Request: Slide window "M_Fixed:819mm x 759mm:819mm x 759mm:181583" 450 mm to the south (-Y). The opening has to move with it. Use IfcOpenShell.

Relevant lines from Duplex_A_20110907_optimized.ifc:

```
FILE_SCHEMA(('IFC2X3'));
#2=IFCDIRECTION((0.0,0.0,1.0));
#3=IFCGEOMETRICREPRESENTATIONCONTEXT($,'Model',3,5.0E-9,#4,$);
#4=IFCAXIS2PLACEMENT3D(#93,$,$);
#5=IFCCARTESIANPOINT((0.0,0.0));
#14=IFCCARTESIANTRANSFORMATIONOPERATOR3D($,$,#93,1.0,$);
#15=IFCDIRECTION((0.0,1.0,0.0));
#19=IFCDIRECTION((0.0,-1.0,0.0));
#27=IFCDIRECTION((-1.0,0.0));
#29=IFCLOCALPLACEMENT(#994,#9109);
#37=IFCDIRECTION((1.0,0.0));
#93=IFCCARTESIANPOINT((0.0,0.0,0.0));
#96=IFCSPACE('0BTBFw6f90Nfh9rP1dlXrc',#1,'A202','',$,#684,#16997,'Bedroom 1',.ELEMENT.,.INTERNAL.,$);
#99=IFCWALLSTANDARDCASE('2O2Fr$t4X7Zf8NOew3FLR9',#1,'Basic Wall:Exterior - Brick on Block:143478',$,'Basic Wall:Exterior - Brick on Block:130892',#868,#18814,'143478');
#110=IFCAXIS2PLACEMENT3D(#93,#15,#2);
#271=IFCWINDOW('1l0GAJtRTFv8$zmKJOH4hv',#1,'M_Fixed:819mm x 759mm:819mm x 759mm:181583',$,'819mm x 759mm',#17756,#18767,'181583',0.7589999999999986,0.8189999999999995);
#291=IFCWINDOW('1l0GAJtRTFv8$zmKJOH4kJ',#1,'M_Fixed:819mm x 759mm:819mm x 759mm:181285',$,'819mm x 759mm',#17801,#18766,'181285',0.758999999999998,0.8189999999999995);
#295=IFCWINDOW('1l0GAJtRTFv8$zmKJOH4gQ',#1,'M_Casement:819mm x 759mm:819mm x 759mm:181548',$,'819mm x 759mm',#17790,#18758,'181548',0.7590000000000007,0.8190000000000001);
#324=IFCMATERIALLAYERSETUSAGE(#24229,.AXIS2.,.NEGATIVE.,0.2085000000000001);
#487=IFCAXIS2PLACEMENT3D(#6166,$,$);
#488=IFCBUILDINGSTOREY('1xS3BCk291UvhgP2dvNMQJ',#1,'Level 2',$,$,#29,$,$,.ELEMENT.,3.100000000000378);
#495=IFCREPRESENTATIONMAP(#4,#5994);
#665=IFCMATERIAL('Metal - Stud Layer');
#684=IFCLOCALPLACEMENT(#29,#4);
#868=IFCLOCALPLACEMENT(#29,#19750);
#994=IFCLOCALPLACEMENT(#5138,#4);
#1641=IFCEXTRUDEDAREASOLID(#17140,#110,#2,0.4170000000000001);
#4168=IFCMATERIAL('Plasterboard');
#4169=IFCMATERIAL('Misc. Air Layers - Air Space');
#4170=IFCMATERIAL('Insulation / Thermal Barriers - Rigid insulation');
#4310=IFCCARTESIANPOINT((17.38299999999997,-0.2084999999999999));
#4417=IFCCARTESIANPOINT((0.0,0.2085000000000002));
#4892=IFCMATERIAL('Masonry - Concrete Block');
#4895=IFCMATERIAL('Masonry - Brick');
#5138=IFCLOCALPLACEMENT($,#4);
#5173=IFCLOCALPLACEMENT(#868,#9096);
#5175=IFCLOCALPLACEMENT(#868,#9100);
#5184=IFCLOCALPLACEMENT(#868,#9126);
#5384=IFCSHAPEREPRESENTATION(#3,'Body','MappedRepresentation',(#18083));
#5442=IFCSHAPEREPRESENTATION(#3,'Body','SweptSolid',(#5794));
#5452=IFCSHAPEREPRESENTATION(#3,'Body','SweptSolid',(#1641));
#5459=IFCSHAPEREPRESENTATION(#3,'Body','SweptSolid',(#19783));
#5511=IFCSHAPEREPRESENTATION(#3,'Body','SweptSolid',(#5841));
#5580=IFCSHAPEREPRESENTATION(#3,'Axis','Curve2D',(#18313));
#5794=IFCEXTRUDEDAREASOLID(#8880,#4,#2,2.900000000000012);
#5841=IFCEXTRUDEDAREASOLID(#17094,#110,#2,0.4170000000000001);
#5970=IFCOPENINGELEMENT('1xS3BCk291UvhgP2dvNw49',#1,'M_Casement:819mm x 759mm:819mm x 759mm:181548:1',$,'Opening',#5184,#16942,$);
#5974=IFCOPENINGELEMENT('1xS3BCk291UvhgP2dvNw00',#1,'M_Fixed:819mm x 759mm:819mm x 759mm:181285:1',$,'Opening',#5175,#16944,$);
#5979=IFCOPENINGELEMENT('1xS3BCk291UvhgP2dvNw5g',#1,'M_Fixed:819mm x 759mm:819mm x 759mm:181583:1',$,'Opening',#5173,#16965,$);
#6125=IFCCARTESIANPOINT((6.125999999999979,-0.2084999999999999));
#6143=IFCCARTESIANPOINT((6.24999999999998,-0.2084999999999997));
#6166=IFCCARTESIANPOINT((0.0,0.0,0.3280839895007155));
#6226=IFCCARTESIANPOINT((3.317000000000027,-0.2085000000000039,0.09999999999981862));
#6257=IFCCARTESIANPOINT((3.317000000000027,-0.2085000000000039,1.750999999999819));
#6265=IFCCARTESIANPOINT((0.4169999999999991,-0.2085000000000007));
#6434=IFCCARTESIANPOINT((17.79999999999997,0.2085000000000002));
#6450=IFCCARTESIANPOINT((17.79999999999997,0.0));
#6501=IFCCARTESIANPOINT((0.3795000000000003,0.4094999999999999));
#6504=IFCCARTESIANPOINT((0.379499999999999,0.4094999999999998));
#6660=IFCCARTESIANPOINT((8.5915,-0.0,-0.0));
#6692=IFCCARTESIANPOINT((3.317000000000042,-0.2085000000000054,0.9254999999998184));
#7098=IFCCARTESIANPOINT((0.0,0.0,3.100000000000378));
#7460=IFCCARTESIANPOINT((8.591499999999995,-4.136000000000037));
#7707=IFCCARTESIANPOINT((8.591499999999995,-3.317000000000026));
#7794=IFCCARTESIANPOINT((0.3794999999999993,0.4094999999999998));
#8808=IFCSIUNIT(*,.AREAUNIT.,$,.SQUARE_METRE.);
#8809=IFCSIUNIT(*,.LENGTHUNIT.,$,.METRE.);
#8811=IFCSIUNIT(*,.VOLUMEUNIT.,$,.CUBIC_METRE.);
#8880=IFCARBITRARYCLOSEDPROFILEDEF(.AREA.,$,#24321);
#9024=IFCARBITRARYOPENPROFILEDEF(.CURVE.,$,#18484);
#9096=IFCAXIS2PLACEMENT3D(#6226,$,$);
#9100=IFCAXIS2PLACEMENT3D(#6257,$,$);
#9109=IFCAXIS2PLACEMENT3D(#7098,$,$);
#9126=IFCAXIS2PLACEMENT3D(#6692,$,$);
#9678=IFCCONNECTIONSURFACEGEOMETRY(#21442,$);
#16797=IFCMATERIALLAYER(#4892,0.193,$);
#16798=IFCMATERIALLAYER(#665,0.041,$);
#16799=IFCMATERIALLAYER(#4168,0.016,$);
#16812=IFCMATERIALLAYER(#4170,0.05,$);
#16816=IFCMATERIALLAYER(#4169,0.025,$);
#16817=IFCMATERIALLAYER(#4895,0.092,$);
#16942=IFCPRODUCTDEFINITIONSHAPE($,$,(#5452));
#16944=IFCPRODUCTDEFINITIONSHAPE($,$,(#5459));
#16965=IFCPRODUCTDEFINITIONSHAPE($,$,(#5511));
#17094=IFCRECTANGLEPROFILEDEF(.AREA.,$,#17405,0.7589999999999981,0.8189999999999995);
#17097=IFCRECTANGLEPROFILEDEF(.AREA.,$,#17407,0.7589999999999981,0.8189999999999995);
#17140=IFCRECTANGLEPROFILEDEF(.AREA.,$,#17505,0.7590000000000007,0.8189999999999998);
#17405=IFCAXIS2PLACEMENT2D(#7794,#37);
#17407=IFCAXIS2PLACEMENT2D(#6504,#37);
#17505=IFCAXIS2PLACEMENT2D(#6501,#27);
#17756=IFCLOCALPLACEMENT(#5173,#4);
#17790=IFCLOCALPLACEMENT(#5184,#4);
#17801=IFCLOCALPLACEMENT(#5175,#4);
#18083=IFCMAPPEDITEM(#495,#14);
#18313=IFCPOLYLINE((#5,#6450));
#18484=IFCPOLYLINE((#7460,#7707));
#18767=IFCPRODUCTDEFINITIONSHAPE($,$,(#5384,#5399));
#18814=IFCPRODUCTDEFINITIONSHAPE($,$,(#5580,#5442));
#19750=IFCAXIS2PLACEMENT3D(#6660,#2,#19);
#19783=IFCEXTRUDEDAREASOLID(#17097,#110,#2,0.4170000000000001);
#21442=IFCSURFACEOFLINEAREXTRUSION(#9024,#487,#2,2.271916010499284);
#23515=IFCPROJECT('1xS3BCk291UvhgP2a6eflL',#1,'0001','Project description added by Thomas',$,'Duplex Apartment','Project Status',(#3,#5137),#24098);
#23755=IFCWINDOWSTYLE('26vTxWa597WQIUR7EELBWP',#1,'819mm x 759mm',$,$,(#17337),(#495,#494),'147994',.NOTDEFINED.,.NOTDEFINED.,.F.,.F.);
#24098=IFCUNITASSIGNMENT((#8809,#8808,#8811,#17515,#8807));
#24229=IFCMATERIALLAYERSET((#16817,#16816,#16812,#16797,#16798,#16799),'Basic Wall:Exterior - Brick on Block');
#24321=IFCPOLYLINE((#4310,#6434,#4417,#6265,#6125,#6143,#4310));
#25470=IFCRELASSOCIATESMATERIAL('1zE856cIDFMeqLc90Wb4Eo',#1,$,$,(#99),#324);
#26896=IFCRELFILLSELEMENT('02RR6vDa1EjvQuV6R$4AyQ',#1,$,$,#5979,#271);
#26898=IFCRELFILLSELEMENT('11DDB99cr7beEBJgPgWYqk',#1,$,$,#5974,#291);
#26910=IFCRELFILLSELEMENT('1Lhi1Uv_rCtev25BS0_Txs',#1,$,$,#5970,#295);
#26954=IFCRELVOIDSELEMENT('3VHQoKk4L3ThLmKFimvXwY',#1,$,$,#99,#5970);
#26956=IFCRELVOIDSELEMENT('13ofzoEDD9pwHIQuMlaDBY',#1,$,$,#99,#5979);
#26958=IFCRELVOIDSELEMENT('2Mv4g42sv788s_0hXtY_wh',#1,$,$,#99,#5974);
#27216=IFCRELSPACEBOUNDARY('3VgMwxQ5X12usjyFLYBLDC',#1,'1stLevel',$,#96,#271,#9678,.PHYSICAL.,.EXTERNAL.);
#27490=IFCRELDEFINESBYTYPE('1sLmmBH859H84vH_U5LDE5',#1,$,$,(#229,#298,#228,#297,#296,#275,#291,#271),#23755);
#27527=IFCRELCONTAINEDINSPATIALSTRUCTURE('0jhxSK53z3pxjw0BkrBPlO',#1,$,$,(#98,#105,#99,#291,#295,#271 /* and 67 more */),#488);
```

```python
import numpy as np
import ifcopenshell
import ifcopenshell.api.geometry
import ifcopenshell.util.placement
import ifcopenshell.util.unit

model = ifcopenshell.open("Duplex_A_20110907_optimized.ifc")
unit_scale = ifcopenshell.util.unit.calculate_unit_scale(model)

window = model.by_id(271)
opening = window.FillsVoids[0].RelatingOpeningElement
wall = opening.VoidsElements[0].RelatingBuildingElement

wall_matrix = ifcopenshell.util.placement.get_local_placement(wall.ObjectPlacement)
shift = wall_matrix[:3, 0] * 0.45 / unit_scale
before = ifcopenshell.util.placement.get_local_placement(window.ObjectPlacement)[:3, 3].copy()

# The window is placed relative to its opening, so it follows when the opening moves.
matrix = ifcopenshell.util.placement.get_local_placement(opening.ObjectPlacement)
matrix[:3, 3] += shift
ifcopenshell.api.geometry.edit_object_placement(
    model, product=opening, matrix=matrix, is_si=False, should_transform_children=True
)

# Space boundary surfaces are stored in each space's coordinates; move them too.
for rel in window.ProvidesBoundaries:
    if not rel.ConnectionGeometry:
        continue
    surface = rel.ConnectionGeometry.SurfaceOnRelatingElement
    space_matrix = ifcopenshell.util.placement.get_local_placement(rel.RelatingSpace.ObjectPlacement)
    point = np.array(surface.Position.Location.Coordinates) + space_matrix[:3, :3].T @ shift
    surface.Position = model.createIfcAxis2Placement3D(
        model.createIfcCartesianPoint(point.tolist()), surface.Position.Axis, surface.Position.RefDirection
    )

after = ifcopenshell.util.placement.get_local_placement(window.ObjectPlacement)[:3, 3]
print("window moved by", (after - before).round(3) + 0.0)

model.write("Duplex_A_20110907_optimized_v2.ifc")
```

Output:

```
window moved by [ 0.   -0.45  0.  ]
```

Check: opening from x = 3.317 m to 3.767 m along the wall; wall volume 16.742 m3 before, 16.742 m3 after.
